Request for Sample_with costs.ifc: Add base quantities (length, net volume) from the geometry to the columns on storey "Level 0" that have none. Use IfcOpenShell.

First a look at what the model holds.

```python
import ifcopenshell
import ifcopenshell.util.element
import ifcopenshell.util.unit

model = ifcopenshell.open("Sample_with costs.ifc")
print(model.schema)
for unit_type in ("LENGTHUNIT", "AREAUNIT", "VOLUMEUNIT"):
    print(unit_type, ifcopenshell.util.unit.calculate_unit_scale(model, unit_type))
storey = next(s for s in model.by_type("IfcBuildingStorey") if s.Name == "Level 0")
columns = [e for e in ifcopenshell.util.element.get_decomposition(storey) if e.is_a("IfcColumn")]
for e in sorted(columns, key=lambda e: e.id()):
    print(e.id(), e.is_a(), e.Name, list(ifcopenshell.util.element.get_psets(e, qtos_only=True)), sep=" | ")
```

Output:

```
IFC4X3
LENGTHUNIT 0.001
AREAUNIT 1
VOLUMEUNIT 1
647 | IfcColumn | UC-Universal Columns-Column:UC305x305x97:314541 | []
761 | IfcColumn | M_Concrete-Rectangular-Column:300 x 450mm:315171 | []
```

```python
import ifcopenshell
import ifcopenshell.api.pset
import ifcopenshell.geom
import ifcopenshell.util.element
import ifcopenshell.util.shape
import ifcopenshell.util.unit

model = ifcopenshell.open("Sample_with costs.ifc")
unit_scale = ifcopenshell.util.unit.calculate_unit_scale(model)
volume_scale = ifcopenshell.util.unit.calculate_unit_scale(model, "VOLUMEUNIT")
settings = ifcopenshell.geom.settings()

storey = next(s for s in model.by_type("IfcBuildingStorey") if s.Name == "Level 0")
columns = [e for e in ifcopenshell.util.element.get_decomposition(storey) if e.is_a("IfcColumn")]

for e in sorted(columns, key=lambda e: e.id()):
    if ifcopenshell.util.element.get_psets(e, qtos_only=True, should_inherit=False):
        continue
    # Geometry comes back in metres, in the element's own axes.
    shape = ifcopenshell.geom.create_shape(settings, e)
    values = {
        "Length": ifcopenshell.util.shape.get_z(shape.geometry) / unit_scale,
        "NetVolume": ifcopenshell.util.shape.get_volume(shape.geometry) / volume_scale,
    }
    qto = ifcopenshell.api.pset.add_qto(model, product=e, name="Qto_ColumnBaseQuantities")
    ifcopenshell.api.pset.edit_qto(model, qto=qto, properties=values)
    print(e.id(), {k: round(v, 3) for k, v in values.items()})

model.write("Sample_with costs_updated.ifc")
```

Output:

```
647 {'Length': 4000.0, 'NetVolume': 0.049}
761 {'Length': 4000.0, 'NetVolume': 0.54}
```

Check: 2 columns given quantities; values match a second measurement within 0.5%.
